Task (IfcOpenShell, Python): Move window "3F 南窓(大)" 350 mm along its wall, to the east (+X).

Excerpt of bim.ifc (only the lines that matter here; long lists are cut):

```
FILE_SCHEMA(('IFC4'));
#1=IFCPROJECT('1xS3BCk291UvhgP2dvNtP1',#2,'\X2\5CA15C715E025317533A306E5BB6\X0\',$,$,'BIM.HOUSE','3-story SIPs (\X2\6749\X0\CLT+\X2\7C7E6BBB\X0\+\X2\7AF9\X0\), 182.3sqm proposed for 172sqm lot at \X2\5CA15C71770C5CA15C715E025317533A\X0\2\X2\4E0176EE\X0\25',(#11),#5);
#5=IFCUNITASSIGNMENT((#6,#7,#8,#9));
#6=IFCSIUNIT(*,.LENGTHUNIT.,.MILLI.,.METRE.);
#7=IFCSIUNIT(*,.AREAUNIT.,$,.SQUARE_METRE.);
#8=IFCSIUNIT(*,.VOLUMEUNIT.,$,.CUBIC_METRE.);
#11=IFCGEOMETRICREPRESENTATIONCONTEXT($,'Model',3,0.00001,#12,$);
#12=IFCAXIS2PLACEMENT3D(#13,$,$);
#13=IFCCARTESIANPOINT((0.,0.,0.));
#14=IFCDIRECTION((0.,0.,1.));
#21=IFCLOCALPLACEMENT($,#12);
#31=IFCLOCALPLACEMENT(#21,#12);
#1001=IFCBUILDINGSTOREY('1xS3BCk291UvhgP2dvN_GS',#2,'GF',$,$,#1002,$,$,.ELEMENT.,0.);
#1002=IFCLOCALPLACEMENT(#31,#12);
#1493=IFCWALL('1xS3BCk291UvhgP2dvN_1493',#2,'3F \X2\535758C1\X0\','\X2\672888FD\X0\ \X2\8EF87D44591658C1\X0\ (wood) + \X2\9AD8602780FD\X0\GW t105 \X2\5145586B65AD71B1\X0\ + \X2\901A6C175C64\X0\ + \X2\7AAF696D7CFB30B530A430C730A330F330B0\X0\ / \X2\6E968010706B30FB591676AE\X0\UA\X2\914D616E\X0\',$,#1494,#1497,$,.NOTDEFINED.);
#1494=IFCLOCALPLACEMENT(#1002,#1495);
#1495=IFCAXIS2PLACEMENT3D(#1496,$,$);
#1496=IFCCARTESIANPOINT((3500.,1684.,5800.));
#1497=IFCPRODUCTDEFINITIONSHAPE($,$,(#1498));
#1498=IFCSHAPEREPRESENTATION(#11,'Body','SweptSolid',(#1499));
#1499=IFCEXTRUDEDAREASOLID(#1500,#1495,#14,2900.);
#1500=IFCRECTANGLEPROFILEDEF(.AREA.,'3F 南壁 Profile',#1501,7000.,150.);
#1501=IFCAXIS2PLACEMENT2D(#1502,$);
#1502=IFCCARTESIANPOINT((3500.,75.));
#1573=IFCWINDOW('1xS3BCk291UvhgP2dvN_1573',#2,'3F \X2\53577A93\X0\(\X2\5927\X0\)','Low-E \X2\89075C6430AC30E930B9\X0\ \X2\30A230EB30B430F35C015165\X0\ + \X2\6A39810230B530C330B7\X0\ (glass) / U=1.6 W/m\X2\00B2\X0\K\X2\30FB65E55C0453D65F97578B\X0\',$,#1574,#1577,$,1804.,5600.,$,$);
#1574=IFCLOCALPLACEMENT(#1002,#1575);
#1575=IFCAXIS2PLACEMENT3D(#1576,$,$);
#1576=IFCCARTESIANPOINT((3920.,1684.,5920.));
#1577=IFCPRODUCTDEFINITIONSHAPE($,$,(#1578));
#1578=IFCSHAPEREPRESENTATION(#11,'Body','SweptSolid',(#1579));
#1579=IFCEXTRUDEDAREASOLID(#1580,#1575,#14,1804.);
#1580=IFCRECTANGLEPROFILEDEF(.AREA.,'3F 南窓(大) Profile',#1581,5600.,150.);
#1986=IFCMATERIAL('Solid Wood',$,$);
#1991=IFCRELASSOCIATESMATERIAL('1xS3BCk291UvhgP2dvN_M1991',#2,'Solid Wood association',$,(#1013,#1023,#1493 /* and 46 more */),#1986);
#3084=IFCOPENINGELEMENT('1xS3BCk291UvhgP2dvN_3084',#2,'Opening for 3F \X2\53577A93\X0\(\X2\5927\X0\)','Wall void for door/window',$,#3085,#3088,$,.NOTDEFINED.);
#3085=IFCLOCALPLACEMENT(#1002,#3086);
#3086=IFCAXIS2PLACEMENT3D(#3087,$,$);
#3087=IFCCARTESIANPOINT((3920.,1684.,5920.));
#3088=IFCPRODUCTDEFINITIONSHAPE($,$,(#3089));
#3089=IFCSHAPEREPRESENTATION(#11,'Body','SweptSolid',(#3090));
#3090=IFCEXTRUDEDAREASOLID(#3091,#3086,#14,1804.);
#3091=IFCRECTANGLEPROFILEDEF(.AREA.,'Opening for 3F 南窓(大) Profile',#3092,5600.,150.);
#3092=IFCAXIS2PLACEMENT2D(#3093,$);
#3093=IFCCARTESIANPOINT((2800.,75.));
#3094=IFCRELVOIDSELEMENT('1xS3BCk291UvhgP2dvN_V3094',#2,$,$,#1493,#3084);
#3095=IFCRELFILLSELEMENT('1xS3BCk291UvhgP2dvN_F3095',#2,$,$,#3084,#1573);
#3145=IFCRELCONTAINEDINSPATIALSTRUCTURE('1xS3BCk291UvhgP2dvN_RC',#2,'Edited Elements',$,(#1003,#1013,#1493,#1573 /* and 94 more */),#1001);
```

```python
import ifcopenshell
import ifcopenshell.api.geometry
import ifcopenshell.util.placement

model = ifcopenshell.open("bim.ifc")

window = model.by_guid("1xS3BCk291UvhgP2dvN_1573")
opening = window.FillsVoids[0].RelatingOpeningElement
wall = opening.VoidsElements[0].RelatingBuildingElement

wall_matrix = ifcopenshell.util.placement.get_local_placement(wall.ObjectPlacement)
shift = wall_matrix[:3, 0] * 350.0
before = ifcopenshell.util.placement.get_local_placement(window.ObjectPlacement)[:3, 3].copy()

# The window is not placed relative to its opening, so move both.
for product in (opening, window):
    matrix = ifcopenshell.util.placement.get_local_placement(product.ObjectPlacement)
    matrix[:3, 3] += shift
    ifcopenshell.api.geometry.edit_object_placement(model, product=product, matrix=matrix, is_si=False)

after = ifcopenshell.util.placement.get_local_placement(window.ObjectPlacement)[:3, 3]
print("window moved by", (after - before).round(3) + 0.0)

model.write("bim_v2.ifc")
```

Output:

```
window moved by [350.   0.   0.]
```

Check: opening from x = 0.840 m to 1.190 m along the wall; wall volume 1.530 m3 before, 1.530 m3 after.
